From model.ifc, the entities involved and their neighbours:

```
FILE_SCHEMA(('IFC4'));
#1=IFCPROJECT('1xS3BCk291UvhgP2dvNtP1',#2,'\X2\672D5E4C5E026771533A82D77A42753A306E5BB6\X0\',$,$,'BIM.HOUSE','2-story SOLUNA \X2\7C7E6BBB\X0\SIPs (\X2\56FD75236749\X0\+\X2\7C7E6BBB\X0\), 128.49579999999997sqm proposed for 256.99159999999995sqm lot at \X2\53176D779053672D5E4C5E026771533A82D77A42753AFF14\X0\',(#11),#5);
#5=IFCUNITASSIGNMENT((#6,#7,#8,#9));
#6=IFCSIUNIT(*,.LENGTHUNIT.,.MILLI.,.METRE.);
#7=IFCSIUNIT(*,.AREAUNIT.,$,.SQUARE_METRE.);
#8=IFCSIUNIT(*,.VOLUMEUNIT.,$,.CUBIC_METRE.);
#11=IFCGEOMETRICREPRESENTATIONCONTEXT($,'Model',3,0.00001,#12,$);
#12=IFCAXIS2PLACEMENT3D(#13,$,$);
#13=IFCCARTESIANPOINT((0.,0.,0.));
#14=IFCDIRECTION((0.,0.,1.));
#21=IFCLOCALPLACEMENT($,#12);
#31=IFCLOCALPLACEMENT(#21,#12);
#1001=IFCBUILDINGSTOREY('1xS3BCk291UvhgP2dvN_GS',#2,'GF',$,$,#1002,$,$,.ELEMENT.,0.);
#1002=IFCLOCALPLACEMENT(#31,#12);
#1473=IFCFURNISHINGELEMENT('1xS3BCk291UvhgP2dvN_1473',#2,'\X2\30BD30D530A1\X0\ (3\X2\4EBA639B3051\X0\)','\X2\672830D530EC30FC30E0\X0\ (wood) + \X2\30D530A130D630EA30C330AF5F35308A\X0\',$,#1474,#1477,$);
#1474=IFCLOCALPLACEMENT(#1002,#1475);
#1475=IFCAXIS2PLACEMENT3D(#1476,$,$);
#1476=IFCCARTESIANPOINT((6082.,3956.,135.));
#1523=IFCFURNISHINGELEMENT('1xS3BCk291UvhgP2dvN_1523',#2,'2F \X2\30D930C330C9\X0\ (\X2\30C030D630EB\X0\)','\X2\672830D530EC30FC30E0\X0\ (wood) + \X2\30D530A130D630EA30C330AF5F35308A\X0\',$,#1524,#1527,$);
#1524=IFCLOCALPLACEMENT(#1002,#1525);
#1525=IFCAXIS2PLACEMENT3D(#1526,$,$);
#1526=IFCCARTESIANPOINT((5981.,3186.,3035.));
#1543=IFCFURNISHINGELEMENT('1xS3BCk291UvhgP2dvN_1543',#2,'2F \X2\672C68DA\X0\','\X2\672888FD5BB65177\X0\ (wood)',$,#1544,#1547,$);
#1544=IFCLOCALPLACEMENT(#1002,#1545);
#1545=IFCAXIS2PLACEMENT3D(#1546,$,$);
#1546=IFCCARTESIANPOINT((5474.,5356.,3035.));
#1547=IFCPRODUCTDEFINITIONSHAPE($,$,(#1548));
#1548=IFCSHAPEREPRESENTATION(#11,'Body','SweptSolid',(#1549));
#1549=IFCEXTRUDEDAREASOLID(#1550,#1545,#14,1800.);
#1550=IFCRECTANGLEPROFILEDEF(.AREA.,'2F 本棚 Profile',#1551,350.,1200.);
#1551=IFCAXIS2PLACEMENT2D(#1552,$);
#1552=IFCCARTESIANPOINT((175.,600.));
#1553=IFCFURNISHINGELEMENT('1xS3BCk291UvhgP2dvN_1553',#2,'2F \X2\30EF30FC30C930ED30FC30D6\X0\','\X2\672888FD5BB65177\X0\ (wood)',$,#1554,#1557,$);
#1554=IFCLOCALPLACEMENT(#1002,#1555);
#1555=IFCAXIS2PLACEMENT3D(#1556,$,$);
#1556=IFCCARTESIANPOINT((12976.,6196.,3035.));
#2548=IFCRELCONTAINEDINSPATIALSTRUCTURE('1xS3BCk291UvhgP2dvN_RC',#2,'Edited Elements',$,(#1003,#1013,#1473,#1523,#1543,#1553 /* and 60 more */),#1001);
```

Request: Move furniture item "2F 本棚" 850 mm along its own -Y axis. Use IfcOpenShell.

```python
import ifcopenshell
import ifcopenshell.api.geometry
import ifcopenshell.util.placement
import ifcopenshell.util.unit

model = ifcopenshell.open("model.ifc")
unit_scale = ifcopenshell.util.unit.calculate_unit_scale(model)

item = model.by_guid("1xS3BCk291UvhgP2dvN_1543")
matrix = ifcopenshell.util.placement.get_local_placement(item.ObjectPlacement)
matrix[:3, 3] -= matrix[:3, 1] * 0.85 / unit_scale
ifcopenshell.api.geometry.edit_object_placement(model, product=item, matrix=matrix, is_si=False)

print(ifcopenshell.util.placement.get_local_placement(item.ObjectPlacement).round(3) + 0.0)

model.write("model_v2.ifc")
```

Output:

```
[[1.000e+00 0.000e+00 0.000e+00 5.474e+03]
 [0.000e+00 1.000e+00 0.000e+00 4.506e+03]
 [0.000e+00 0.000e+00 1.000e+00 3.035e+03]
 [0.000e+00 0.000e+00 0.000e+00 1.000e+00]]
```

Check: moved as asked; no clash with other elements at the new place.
